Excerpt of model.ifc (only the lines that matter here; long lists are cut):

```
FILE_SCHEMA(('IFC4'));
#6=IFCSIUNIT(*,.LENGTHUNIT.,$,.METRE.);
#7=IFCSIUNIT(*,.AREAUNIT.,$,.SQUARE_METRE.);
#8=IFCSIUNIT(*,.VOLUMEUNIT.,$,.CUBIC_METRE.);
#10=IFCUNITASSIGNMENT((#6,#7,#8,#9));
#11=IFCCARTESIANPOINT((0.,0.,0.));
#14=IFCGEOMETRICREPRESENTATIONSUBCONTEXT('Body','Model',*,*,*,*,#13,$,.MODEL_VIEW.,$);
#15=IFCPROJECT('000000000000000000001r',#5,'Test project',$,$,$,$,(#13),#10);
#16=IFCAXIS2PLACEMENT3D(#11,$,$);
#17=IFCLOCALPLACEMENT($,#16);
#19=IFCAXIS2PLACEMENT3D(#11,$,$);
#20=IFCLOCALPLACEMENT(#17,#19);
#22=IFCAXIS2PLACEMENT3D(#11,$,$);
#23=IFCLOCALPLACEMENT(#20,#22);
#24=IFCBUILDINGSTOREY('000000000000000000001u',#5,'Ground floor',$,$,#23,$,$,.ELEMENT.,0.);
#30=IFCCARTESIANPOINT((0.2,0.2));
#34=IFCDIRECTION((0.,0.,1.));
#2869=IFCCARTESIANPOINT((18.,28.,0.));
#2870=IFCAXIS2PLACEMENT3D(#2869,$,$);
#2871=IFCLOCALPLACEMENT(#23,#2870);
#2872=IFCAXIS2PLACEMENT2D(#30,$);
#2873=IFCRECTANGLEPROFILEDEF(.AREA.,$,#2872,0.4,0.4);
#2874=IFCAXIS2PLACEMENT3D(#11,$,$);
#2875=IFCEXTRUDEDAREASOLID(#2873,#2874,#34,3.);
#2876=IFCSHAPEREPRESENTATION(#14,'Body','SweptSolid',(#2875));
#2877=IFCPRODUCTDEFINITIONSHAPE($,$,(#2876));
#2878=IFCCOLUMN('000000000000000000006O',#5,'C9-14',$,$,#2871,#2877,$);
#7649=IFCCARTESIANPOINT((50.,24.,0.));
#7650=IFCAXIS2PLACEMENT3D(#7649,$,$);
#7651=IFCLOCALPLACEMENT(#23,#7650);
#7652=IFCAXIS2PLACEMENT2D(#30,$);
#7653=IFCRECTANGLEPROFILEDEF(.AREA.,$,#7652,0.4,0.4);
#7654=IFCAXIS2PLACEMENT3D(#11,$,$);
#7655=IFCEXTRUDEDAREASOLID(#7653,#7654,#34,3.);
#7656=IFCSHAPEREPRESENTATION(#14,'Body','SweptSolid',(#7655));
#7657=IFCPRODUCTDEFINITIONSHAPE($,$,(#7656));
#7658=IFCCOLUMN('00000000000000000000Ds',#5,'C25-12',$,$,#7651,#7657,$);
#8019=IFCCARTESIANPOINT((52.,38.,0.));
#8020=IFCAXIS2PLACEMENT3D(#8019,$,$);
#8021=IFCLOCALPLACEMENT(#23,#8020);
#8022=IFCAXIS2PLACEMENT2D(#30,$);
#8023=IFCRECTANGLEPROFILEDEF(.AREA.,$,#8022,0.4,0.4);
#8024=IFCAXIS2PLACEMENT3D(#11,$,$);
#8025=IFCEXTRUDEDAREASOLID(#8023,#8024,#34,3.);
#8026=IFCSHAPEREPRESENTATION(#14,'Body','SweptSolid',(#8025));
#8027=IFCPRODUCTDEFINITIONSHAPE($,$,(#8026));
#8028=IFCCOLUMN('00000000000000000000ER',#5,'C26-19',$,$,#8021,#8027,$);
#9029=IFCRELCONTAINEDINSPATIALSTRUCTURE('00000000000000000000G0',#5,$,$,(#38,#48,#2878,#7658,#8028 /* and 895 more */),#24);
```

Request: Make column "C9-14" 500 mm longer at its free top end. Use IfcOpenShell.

```python
import ifcopenshell
import ifcopenshell.util.representation
import ifcopenshell.util.unit

model = ifcopenshell.open("model.ifc")
unit_scale = ifcopenshell.util.unit.calculate_unit_scale(model)

member = model.by_guid("000000000000000000006O")
change = 0.5 / unit_scale

# The extrusion runs towards the end named, so only its depth changes.
body = ifcopenshell.util.representation.get_representation(member, "Model", "Body")
solid = body.Items[0]
old_length = solid.Depth
solid.Depth += change

print(f"length {old_length:g} -> {solid.Depth:g}")

model.write("model_rev.ifc")
```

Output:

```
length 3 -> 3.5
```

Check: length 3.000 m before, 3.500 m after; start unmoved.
